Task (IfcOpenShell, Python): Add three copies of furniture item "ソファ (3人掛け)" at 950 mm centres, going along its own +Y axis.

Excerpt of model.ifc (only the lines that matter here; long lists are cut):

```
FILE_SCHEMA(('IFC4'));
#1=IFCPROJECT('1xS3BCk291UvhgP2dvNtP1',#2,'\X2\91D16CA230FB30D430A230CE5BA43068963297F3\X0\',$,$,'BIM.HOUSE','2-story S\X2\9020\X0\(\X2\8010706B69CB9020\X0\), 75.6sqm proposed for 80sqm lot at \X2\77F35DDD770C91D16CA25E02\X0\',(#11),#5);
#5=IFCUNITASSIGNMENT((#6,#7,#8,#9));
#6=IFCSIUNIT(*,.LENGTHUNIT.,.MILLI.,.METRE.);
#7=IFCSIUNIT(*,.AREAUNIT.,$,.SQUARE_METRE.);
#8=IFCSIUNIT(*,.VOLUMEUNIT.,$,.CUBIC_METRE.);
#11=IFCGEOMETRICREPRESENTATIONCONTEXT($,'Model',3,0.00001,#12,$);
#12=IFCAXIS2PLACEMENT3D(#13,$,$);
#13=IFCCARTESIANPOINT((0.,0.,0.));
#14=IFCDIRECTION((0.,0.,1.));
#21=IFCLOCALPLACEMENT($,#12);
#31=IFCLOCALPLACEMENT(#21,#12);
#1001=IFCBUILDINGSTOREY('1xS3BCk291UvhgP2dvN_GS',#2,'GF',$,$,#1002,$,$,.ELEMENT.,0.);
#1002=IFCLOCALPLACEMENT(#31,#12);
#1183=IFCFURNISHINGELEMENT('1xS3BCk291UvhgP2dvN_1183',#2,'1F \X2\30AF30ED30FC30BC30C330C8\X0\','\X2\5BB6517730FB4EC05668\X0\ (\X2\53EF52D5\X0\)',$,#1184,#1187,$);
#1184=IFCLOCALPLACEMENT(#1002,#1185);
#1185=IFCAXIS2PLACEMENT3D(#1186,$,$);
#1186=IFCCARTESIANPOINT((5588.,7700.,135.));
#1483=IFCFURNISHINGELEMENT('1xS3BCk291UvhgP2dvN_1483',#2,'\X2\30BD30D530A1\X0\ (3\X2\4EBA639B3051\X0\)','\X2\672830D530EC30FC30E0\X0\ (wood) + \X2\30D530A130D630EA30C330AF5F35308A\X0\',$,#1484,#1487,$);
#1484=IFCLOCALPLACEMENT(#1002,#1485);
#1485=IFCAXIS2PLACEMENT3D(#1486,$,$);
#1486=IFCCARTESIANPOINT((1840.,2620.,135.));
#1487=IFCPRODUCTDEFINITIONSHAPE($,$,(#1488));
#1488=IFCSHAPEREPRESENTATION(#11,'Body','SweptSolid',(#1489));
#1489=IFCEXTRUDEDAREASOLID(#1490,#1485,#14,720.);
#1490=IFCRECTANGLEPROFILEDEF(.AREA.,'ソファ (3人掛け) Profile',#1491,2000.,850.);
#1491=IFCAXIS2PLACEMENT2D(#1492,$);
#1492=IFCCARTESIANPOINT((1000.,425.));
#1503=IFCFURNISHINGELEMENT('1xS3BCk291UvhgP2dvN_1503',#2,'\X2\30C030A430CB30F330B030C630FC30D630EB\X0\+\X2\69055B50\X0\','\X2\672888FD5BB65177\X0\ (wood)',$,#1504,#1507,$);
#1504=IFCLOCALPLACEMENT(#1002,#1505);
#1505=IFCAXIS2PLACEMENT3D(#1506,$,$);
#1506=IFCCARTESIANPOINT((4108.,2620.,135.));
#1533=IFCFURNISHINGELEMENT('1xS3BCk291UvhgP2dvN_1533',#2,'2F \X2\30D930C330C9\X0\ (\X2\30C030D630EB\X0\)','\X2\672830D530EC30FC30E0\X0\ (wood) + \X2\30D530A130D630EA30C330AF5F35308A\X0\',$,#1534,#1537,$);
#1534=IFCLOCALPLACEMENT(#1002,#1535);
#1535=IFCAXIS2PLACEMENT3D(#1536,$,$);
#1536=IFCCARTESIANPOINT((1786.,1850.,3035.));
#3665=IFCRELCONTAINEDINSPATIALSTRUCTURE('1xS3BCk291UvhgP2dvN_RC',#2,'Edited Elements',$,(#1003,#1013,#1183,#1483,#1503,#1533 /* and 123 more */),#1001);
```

```python
import ifcopenshell
import ifcopenshell.api.geometry
import ifcopenshell.api.root
import ifcopenshell.util.element
import ifcopenshell.util.placement
import ifcopenshell.util.unit

model = ifcopenshell.open("model.ifc")
unit_scale = ifcopenshell.util.unit.calculate_unit_scale(model)


def reuse_history(source, copy):
    """copy_class also copies each property set's owner history, people and application; keep the originals."""
    for rel in copy.IsDefinedBy:
        if rel.is_a("IfcRelDefinesByProperties") and (history := rel.RelatingPropertyDefinition.OwnerHistory):
            rel.RelatingPropertyDefinition.OwnerHistory = source.OwnerHistory
            ifcopenshell.util.element.remove_deep2(model, history)


source = model.by_id(1483)
base = ifcopenshell.util.placement.get_local_placement(source.ObjectPlacement)
step = base[:3, 1] * 0.95 / unit_scale

for i in range(1, 4):
    copy = ifcopenshell.api.root.copy_class(model, product=source)
    copy.Representation = ifcopenshell.util.element.copy_deep(
        model, source.Representation, exclude=["IfcGeometricRepresentationContext", "IfcRepresentationMap"]
    )
    reuse_history(source, copy)
    matrix = base.copy()
    matrix[:3, 3] += i * step
    print("added at", matrix[:3, 3].round(3) + 0.0)
    ifcopenshell.api.geometry.edit_object_placement(model, product=copy, matrix=matrix, is_si=False)

model.write("model_v2.ifc")
```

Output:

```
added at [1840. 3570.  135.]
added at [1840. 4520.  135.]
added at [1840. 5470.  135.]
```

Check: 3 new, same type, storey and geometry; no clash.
